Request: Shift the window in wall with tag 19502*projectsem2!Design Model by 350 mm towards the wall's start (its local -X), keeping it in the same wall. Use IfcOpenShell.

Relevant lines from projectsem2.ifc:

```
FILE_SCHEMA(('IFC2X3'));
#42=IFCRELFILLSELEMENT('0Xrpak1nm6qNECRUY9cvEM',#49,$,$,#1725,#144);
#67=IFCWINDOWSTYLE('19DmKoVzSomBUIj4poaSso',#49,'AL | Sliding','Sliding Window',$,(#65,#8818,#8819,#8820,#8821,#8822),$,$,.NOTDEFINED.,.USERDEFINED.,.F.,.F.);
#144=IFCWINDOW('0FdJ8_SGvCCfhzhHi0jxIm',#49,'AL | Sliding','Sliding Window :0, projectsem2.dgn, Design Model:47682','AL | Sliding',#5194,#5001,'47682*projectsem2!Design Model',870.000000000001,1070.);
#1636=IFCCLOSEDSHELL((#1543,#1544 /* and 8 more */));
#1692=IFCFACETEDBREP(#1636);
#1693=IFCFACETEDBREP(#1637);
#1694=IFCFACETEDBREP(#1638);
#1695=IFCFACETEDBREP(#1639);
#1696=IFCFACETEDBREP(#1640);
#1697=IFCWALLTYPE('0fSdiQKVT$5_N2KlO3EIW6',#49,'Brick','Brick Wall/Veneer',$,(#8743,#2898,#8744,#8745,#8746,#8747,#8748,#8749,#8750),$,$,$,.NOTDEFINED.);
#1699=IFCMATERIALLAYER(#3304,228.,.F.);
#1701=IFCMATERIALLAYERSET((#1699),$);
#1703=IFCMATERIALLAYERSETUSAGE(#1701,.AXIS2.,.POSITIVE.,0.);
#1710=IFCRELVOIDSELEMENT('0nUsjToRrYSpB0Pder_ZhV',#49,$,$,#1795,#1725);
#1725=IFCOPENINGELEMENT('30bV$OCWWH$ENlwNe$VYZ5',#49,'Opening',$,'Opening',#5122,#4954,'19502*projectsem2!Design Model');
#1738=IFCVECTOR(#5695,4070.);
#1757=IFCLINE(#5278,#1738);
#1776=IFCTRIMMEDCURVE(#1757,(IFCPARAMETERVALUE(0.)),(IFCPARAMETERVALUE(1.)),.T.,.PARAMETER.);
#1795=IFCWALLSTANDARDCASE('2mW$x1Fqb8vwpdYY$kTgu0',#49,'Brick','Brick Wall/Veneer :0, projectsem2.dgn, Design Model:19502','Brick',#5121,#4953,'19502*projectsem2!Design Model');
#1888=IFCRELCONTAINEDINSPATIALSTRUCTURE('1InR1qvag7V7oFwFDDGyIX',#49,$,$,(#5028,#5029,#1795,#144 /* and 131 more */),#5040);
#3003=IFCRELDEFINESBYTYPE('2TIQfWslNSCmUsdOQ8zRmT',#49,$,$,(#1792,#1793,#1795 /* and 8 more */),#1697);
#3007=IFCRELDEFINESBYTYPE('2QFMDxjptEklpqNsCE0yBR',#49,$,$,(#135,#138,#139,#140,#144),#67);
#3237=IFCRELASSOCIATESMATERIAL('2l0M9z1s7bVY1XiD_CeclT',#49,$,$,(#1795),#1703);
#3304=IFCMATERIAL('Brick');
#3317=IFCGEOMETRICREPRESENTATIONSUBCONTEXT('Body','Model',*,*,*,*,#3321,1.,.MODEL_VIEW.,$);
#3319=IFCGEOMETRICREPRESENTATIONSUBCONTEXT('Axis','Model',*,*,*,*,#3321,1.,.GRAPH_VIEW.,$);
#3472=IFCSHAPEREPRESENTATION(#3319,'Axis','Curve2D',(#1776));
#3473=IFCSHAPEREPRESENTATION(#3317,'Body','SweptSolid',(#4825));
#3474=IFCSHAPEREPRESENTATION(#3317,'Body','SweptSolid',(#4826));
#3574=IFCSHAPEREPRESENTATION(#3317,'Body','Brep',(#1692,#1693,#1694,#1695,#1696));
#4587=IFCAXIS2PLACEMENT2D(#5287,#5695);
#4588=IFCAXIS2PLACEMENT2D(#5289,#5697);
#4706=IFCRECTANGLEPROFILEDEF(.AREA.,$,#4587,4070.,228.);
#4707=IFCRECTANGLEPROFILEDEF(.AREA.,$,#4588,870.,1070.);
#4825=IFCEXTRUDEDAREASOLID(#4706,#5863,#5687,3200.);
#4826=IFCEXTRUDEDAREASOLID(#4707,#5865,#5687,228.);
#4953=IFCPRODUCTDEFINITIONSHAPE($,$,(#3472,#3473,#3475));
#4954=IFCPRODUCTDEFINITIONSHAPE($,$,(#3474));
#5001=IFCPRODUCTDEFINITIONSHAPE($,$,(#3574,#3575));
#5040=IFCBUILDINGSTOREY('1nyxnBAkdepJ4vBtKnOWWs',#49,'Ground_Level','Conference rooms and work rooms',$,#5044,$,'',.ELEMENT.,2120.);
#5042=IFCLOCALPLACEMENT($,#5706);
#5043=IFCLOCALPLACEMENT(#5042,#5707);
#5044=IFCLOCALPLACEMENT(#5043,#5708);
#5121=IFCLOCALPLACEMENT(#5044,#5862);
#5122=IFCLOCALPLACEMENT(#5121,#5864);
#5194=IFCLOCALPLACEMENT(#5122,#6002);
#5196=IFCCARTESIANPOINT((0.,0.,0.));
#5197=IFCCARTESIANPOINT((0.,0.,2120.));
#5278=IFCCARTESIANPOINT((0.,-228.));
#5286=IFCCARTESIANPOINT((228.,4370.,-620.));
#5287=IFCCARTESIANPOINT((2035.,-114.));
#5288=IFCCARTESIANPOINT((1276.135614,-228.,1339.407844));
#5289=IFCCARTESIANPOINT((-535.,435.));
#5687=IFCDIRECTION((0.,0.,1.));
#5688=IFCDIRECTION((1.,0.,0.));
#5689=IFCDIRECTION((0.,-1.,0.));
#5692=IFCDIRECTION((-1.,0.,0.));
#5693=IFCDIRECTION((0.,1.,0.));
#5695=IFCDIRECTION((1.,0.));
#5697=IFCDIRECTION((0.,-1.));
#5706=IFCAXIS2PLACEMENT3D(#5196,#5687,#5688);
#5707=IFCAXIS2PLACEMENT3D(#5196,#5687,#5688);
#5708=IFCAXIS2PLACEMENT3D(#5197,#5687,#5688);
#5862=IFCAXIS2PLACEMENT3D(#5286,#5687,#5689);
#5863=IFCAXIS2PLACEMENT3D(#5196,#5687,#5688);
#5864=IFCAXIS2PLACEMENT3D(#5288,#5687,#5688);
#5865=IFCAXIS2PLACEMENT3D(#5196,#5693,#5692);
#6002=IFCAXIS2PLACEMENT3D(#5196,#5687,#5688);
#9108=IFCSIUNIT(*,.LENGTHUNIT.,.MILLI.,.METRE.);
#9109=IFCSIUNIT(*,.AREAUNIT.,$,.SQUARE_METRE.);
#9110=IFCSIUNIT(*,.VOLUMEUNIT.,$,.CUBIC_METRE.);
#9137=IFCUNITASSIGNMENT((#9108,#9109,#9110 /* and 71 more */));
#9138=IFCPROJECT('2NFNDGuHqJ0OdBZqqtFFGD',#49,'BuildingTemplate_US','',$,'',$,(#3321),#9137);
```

```python
import ifcopenshell
import ifcopenshell.api.geometry
import ifcopenshell.util.placement

model = ifcopenshell.open("projectsem2.ifc")

window = model.by_guid("0FdJ8_SGvCCfhzhHi0jxIm")
opening = window.FillsVoids[0].RelatingOpeningElement
wall = opening.VoidsElements[0].RelatingBuildingElement

wall_matrix = ifcopenshell.util.placement.get_local_placement(wall.ObjectPlacement)
shift = wall_matrix[:3, 0] * -350.0
before = ifcopenshell.util.placement.get_local_placement(window.ObjectPlacement)[:3, 3].copy()

# The window is placed relative to its opening, so it follows when the opening moves.
matrix = ifcopenshell.util.placement.get_local_placement(opening.ObjectPlacement)
matrix[:3, 3] += shift
ifcopenshell.api.geometry.edit_object_placement(
    model, product=opening, matrix=matrix, is_si=False, should_transform_children=True
)

after = ifcopenshell.util.placement.get_local_placement(window.ObjectPlacement)[:3, 3]
print("window moved by", (after - before).round(3) + 0.0)

model.write("projectsem2_v2.ifc")
```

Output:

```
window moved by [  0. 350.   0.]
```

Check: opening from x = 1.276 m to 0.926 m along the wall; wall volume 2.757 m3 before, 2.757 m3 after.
